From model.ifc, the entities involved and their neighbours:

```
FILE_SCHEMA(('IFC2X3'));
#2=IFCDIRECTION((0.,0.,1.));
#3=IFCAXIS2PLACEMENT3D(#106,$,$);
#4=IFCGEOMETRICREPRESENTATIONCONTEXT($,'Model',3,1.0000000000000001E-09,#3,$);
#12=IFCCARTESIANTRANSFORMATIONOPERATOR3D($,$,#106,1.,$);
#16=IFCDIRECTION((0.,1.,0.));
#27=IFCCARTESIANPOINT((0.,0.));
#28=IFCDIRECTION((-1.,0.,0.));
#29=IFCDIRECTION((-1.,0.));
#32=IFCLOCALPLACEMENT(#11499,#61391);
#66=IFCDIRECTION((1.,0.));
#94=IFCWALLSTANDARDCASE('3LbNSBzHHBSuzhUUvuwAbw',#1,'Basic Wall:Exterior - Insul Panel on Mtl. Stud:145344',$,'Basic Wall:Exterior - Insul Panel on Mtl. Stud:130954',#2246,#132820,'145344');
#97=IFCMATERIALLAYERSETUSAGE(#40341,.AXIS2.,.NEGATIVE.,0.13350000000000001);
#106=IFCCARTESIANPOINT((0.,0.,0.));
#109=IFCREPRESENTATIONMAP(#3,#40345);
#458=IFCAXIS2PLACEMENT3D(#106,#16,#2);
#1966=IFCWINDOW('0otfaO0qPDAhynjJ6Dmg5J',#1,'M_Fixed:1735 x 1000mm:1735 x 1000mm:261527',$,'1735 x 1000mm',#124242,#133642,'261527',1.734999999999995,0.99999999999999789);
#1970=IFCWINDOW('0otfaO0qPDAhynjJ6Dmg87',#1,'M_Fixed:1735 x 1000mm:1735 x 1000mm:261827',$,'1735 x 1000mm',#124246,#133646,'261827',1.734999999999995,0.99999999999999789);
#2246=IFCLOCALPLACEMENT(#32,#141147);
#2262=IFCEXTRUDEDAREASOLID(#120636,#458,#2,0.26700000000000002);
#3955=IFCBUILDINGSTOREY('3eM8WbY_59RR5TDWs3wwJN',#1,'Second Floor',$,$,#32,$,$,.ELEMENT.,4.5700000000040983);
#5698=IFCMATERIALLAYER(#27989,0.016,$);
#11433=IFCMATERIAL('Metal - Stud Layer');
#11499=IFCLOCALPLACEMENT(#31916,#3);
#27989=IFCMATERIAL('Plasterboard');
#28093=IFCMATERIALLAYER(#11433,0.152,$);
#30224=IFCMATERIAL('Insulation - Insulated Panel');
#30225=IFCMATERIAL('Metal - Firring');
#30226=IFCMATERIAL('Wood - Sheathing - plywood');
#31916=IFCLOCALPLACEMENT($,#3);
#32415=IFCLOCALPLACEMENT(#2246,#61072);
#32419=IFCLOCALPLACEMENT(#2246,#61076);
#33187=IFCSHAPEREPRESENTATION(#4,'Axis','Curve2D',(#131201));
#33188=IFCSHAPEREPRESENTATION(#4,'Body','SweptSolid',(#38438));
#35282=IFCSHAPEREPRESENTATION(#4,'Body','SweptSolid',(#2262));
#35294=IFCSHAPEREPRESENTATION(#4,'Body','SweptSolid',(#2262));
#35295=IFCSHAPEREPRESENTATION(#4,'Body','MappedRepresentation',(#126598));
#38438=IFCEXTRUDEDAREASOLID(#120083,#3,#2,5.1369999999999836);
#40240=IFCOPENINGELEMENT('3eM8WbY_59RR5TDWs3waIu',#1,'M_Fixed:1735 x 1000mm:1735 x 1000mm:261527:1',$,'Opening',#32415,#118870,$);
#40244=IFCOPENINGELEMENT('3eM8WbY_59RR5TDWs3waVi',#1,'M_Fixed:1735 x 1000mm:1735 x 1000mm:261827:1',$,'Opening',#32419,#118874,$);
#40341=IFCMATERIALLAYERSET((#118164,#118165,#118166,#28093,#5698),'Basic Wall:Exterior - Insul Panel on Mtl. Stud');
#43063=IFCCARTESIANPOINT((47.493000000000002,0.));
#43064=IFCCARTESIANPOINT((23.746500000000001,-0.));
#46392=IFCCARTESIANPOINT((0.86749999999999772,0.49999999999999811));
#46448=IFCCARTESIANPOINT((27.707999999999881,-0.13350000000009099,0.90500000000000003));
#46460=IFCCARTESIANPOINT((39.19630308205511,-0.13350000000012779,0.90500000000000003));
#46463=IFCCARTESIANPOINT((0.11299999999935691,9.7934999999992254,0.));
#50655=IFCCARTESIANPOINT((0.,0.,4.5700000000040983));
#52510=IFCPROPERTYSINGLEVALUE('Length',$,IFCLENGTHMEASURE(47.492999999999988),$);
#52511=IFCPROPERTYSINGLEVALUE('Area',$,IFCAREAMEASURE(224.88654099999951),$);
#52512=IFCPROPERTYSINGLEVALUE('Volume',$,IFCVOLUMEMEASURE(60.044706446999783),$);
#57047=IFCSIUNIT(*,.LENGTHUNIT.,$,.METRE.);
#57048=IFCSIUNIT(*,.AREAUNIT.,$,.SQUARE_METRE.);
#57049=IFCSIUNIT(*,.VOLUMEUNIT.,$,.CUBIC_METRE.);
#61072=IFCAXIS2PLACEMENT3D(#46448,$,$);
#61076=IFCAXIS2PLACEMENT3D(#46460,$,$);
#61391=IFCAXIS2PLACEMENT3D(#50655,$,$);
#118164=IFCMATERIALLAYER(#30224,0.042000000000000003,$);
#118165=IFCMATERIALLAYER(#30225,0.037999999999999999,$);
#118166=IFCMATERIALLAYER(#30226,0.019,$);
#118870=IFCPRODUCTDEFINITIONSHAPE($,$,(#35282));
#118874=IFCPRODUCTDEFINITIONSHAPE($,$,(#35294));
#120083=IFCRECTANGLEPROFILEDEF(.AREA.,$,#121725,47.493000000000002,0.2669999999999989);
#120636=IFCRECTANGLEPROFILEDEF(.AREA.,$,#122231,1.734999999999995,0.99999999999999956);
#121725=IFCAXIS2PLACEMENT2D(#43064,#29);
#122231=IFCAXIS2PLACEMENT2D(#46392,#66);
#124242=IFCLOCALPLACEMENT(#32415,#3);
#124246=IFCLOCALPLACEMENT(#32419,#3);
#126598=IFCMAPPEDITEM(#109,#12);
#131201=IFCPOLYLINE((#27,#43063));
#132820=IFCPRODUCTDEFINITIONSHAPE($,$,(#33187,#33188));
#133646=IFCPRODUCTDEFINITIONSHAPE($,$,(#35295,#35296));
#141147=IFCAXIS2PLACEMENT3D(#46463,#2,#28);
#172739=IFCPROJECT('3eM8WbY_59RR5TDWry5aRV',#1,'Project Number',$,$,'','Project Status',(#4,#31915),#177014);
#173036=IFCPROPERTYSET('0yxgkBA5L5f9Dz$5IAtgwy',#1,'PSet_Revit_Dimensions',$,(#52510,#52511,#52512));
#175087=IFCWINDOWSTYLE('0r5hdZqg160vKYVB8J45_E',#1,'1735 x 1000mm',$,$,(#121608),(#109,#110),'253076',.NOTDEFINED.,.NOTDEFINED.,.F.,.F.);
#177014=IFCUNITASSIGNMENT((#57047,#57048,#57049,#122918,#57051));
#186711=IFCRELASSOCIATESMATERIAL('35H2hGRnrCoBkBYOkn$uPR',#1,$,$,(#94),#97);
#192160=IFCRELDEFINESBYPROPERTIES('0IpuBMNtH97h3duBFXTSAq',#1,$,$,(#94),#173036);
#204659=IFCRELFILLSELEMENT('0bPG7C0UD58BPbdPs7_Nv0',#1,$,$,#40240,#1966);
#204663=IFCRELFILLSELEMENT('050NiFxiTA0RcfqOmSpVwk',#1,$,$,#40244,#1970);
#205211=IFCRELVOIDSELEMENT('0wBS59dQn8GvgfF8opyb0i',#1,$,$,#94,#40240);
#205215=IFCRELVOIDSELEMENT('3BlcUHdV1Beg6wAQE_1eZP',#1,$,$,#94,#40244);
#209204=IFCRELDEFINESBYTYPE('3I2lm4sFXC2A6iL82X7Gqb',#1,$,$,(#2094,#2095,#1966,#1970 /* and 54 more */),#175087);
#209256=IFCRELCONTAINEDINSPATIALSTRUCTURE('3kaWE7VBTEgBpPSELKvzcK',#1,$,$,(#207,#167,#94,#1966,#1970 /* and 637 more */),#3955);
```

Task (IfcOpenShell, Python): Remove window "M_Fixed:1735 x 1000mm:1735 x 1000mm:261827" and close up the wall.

```python
import ifcopenshell
import ifcopenshell.api.feature
import ifcopenshell.api.pset
import ifcopenshell.api.root
import ifcopenshell.geom
import ifcopenshell.util.element
import ifcopenshell.util.shape
import ifcopenshell.util.unit

model = ifcopenshell.open("model.ifc")
area_scale = ifcopenshell.util.unit.calculate_unit_scale(model, "AREAUNIT")
volume_scale = ifcopenshell.util.unit.calculate_unit_scale(model, "VOLUMEUNIT")
settings = ifcopenshell.geom.settings()


def volume(element):
    """Net volume in cubic metres, openings subtracted."""
    shape = ifcopenshell.geom.create_shape(settings, element)
    return ifcopenshell.util.shape.get_volume(shape.geometry)


window = model.by_guid("0otfaO0qPDAhynjJ6Dmg87")
opening = window.FillsVoids[0].RelatingOpeningElement
wall = opening.VoidsElements[0].RelatingBuildingElement
before = volume(wall)

ifcopenshell.api.root.remove_product(model, product=window)
ifcopenshell.api.feature.remove_feature(model, feature=opening)

after = volume(wall)
thickness = 0.267  # wall thickness in metres

# Update the wall's stored quantities.
pset = model.by_id(ifcopenshell.util.element.get_pset(wall, "PSet_Revit_Dimensions", should_inherit=False)["id"])
ifcopenshell.api.pset.edit_pset(model, pset=pset, properties={
    "Area": model.create_entity("IfcAreaMeasure", after / thickness / area_scale),
    "Volume": model.create_entity("IfcVolumeMeasure", after / volume_scale),
})

print(f"wall volume {before:.3f} -> {after:.3f} m3")

model.write("model_v2.ifc")
```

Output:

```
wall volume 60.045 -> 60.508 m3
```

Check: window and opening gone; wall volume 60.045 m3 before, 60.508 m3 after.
